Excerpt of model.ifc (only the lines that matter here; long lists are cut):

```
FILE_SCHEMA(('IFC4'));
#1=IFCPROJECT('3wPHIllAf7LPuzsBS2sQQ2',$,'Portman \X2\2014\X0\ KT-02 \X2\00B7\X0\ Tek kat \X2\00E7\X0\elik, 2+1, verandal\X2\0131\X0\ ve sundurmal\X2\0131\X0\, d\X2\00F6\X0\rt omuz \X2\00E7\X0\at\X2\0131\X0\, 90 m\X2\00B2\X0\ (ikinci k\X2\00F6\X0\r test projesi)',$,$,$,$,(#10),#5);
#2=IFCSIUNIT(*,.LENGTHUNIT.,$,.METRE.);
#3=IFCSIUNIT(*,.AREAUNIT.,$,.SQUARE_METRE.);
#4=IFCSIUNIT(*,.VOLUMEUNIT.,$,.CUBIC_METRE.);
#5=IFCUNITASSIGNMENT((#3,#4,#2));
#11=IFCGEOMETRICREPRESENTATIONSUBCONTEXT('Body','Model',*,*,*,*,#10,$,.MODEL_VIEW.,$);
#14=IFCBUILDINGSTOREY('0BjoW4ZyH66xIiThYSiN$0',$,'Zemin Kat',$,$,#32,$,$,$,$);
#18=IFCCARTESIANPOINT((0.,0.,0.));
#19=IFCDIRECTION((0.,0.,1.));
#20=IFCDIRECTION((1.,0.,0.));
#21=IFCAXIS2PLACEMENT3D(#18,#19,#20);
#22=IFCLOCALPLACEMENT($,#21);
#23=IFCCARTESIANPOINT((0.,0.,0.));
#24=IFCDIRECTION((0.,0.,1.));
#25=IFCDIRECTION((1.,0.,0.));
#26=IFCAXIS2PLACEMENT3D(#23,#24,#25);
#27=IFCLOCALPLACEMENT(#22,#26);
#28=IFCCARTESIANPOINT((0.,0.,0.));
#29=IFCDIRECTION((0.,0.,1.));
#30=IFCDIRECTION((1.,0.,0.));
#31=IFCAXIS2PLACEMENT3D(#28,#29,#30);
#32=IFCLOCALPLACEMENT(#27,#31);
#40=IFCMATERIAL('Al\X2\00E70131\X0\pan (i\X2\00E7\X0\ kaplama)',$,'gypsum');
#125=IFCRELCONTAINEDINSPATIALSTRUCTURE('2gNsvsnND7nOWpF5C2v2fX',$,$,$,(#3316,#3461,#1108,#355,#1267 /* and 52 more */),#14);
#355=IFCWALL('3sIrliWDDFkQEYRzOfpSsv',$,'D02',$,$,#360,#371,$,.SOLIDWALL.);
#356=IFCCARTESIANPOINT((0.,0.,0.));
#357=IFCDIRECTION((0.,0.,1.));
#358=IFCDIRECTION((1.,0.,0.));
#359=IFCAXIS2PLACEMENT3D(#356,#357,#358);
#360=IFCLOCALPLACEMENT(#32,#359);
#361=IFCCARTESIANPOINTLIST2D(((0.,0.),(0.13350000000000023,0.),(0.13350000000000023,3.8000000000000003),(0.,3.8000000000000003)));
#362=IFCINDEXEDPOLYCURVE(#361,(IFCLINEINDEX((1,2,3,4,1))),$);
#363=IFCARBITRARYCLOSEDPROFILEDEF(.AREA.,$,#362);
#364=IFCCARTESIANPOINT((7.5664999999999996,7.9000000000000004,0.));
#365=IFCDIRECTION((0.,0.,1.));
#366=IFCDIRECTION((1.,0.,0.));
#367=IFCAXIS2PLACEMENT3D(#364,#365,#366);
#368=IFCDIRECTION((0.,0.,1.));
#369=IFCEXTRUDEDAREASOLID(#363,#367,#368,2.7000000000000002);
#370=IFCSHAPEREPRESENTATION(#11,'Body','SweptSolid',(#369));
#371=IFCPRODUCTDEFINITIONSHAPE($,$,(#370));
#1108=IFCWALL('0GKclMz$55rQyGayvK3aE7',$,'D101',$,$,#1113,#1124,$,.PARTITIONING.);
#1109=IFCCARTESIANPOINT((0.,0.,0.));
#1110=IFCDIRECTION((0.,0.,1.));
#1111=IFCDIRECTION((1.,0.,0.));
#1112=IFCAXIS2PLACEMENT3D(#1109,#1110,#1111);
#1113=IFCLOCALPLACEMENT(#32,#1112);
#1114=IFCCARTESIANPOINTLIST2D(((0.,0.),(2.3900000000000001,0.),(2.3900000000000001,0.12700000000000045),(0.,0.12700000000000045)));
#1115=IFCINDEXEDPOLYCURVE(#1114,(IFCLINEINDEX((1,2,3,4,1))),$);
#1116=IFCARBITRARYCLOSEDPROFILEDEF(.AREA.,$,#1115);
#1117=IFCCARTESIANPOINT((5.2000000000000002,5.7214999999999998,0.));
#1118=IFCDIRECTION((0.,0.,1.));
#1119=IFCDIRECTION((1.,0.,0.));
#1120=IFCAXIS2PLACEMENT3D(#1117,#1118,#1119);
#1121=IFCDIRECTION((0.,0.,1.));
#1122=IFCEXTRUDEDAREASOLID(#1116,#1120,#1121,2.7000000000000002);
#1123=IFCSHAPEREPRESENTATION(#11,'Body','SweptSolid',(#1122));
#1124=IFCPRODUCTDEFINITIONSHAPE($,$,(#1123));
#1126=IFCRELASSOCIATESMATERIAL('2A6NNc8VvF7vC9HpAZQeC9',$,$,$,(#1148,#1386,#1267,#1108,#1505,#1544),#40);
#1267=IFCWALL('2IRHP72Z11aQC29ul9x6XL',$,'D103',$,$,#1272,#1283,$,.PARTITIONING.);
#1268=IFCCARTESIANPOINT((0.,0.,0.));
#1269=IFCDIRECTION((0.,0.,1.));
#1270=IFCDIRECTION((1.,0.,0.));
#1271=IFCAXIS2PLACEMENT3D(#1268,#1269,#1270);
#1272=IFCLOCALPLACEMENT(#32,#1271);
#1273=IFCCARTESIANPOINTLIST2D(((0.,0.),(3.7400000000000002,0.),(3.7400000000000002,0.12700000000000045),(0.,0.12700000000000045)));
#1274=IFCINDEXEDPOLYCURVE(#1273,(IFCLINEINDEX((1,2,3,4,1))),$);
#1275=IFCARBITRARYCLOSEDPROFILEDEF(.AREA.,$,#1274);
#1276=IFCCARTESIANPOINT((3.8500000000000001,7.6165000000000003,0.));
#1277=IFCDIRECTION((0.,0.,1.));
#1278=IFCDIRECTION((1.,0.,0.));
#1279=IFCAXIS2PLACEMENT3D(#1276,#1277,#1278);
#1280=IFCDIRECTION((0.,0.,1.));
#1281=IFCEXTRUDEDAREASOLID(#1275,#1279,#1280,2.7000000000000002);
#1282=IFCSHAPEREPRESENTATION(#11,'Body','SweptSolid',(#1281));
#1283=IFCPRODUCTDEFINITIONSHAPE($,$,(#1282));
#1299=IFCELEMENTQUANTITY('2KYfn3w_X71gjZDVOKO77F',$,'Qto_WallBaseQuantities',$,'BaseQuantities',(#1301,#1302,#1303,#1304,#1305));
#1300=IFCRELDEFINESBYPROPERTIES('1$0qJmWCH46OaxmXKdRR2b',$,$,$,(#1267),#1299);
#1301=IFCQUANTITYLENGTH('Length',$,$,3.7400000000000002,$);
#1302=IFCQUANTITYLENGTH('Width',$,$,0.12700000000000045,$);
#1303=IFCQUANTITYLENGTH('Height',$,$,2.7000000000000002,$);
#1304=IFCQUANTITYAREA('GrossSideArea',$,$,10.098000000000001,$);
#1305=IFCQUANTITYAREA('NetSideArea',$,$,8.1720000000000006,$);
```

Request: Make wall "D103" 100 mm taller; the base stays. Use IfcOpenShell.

```python
import ifcopenshell
import ifcopenshell.api.pset
import ifcopenshell.geom
import ifcopenshell.util.element
import ifcopenshell.util.representation
import ifcopenshell.util.shape
import ifcopenshell.util.unit

model = ifcopenshell.open("model.ifc")
unit_scale = ifcopenshell.util.unit.calculate_unit_scale(model)
area_scale = ifcopenshell.util.unit.calculate_unit_scale(model, "AREAUNIT")
settings = ifcopenshell.geom.settings()


def volume(element):
    """Net volume in cubic metres, openings subtracted."""
    shape = ifcopenshell.geom.create_shape(settings, element)
    return ifcopenshell.util.shape.get_volume(shape.geometry)


wall = model.by_guid("2IRHP72Z11aQC29ul9x6XL")
before = volume(wall)

body = ifcopenshell.util.representation.get_representation(wall, "Model", "Body")
solid = body.Items[0]
old_height = solid.Depth
solid.Depth += 0.1 / unit_scale
after = volume(wall)
thickness = 0.127  # wall thickness in metres

# Update the stored height, areas and volumes.
qto = model.by_id(ifcopenshell.util.element.get_pset(wall, "Qto_WallBaseQuantities", should_inherit=False)["id"])
ifcopenshell.api.pset.edit_qto(model, qto=qto, properties={
    "Height": solid.Depth,
    "GrossSideArea": ifcopenshell.util.element.get_pset(wall, "Qto_WallBaseQuantities", "GrossSideArea") * solid.Depth / old_height,
    "NetSideArea": after / thickness / area_scale,
})

print(f"height {old_height:g} -> {solid.Depth:g}, volume {before:.3f} -> {after:.3f} m3")

model.write("model_edited.ifc")
```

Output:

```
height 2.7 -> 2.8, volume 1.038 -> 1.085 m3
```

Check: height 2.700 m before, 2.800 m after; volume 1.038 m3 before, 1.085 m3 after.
